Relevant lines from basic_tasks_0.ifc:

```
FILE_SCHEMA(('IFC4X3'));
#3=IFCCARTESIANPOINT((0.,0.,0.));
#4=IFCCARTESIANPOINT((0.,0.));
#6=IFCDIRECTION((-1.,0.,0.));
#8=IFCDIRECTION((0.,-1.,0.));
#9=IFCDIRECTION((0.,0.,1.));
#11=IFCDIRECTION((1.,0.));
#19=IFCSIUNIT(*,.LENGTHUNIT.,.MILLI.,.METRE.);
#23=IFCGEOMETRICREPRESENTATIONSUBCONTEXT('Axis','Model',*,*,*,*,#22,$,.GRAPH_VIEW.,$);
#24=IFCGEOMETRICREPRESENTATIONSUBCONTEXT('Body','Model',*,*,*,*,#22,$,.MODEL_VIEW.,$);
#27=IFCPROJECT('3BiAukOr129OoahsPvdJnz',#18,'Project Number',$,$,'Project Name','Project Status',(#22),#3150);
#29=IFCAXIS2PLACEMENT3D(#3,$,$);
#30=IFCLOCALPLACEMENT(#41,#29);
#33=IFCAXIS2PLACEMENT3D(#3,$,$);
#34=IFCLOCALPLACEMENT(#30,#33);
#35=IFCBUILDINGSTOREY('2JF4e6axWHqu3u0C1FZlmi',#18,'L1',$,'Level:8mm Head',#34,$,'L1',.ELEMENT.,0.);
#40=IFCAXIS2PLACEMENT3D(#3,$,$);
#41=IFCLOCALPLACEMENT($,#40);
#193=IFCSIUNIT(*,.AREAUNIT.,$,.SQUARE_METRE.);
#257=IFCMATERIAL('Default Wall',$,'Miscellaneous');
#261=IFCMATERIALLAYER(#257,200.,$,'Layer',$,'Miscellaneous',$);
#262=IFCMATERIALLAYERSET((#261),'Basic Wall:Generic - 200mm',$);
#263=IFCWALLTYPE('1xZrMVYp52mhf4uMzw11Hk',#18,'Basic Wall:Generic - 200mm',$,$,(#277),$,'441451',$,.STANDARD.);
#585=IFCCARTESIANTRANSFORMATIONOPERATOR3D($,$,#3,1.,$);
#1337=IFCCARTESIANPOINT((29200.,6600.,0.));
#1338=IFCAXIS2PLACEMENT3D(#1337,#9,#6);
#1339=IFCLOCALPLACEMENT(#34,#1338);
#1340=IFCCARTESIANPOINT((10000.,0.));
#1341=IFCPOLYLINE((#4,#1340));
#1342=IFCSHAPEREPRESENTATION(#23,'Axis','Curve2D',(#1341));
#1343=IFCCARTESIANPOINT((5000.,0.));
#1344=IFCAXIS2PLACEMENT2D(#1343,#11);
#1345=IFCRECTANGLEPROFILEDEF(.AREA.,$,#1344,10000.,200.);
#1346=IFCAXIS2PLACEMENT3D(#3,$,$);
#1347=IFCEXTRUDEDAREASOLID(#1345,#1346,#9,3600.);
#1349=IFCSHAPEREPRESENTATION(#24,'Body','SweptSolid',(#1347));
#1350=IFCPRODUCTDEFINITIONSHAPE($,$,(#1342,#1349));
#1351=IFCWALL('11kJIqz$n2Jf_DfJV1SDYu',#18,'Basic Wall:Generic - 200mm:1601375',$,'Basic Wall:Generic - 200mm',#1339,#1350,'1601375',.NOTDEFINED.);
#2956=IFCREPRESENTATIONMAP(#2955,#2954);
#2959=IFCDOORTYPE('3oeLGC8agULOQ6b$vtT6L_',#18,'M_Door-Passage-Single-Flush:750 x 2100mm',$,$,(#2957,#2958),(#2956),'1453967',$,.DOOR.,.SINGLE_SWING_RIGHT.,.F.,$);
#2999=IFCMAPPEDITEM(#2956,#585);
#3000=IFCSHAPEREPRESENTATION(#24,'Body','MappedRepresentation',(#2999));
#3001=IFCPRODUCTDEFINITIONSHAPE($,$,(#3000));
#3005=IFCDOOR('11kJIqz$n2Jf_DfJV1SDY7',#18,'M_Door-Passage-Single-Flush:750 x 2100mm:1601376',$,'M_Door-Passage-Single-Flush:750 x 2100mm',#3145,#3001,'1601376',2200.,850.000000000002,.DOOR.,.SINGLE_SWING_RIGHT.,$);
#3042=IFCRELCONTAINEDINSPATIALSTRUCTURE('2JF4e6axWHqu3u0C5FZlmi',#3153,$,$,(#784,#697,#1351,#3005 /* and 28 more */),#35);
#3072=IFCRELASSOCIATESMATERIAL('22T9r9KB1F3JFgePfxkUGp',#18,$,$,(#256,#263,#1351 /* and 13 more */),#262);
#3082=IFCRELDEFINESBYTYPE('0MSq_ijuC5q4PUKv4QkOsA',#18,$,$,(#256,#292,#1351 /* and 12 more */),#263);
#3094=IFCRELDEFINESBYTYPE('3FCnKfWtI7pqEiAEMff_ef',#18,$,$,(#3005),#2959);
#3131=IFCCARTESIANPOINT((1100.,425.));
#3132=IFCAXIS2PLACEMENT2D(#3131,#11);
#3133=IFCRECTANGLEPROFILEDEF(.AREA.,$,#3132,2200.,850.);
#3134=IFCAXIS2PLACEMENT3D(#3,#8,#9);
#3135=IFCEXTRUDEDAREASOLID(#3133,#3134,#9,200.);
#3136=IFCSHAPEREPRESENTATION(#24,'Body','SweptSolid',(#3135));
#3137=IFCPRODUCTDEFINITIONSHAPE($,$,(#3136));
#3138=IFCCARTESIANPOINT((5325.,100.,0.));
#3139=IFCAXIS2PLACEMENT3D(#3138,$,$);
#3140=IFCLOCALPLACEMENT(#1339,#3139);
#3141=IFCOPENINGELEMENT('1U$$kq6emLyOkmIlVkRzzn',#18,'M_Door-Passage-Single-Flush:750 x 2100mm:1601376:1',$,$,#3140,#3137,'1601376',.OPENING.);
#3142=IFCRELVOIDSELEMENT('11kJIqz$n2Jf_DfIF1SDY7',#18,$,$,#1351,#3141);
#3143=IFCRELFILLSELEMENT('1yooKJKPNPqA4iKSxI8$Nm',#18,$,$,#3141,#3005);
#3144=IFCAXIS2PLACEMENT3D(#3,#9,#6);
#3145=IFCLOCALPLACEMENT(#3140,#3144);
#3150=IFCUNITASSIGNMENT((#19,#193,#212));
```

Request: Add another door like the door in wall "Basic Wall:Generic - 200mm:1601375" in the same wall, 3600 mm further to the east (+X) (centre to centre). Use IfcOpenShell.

```python
import ifcopenshell
import ifcopenshell.api.feature
import ifcopenshell.api.geometry
import ifcopenshell.api.root
import ifcopenshell.geom
import ifcopenshell.util.element
import ifcopenshell.util.placement
import ifcopenshell.util.shape
import ifcopenshell.util.unit

model = ifcopenshell.open("basic_tasks_0.ifc")
unit_scale = ifcopenshell.util.unit.calculate_unit_scale(model)
settings = ifcopenshell.geom.settings()


def volume(element):
    """Net volume in cubic metres, openings subtracted."""
    shape = ifcopenshell.geom.create_shape(settings, element)
    return ifcopenshell.util.shape.get_volume(shape.geometry)


def reuse_history(source, copy):
    """copy_class also copies each property set's owner history, people and application; keep the originals."""
    for rel in copy.IsDefinedBy:
        if rel.is_a("IfcRelDefinesByProperties") and (history := rel.RelatingPropertyDefinition.OwnerHistory):
            rel.RelatingPropertyDefinition.OwnerHistory = source.OwnerHistory
            ifcopenshell.util.element.remove_deep2(model, history)


door = model.by_guid("11kJIqz$n2Jf_DfJV1SDY7")
opening = door.FillsVoids[0].RelatingOpeningElement
wall = opening.VoidsElements[0].RelatingBuildingElement
before = volume(wall)
shift = ifcopenshell.util.placement.get_local_placement(wall.ObjectPlacement)[:3, 0] * -3.6 / unit_scale

# copy_class copies the void relationship, type, container and properties, but no geometry.
new_opening = ifcopenshell.api.root.copy_class(model, product=opening)
new_opening.Representation = ifcopenshell.util.element.copy_deep(
    model, opening.Representation, exclude=["IfcGeometricRepresentationContext", "IfcRepresentationMap"]
)
new_opening.Name = "M_Door-Passage-Single-Flush:750 x 2100mm"
new_opening.Tag = None
new_door = ifcopenshell.api.root.copy_class(model, product=door)
new_door.Representation = ifcopenshell.util.element.copy_deep(
    model, door.Representation, exclude=["IfcGeometricRepresentationContext", "IfcRepresentationMap"]
)
new_door.Name = "M_Door-Passage-Single-Flush:750 x 2100mm"
new_door.Tag = None
reuse_history(door, new_door)
ifcopenshell.api.feature.add_filling(model, opening=new_opening, element=new_door)

for old, new in ((opening, new_opening), (door, new_door)):
    matrix = ifcopenshell.util.placement.get_local_placement(old.ObjectPlacement)
    matrix[:3, 3] += shift
    ifcopenshell.api.geometry.edit_object_placement(model, product=new, matrix=matrix, is_si=False)

after = volume(wall)

print(f"wall volume {before:.3f} -> {after:.3f} m3")

model.write("basic_tasks_0_v2.ifc")
```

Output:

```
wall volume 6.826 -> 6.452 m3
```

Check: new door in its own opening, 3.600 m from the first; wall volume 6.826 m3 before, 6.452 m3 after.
